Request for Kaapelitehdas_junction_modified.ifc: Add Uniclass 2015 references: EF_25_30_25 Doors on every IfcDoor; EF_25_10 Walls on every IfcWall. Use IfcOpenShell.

First a look at what the model holds.

```python
import ifcopenshell

model = ifcopenshell.open("Kaapelitehdas_junction_modified.ifc")
print(model.schema)
print("classifications:", [c.Name for c in model.by_type("IfcClassification")])
for ifc_class in ("IfcDoor", "IfcRoof", "IfcStair", "IfcWall", "IfcWindow"):
    print(ifc_class, len(model.by_type(ifc_class)))
```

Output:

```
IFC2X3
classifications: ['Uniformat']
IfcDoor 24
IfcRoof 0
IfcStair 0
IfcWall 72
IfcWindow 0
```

```python
import ifcopenshell
import ifcopenshell.api.classification

model = ifcopenshell.open("Kaapelitehdas_junction_modified.ifc")

# IFC2X3 requires Source and Edition and has no link from the project to the system.
system = model.create_entity("IfcClassification", Source="NBS", Edition="2015", Name="Uniclass 2015")

codes = {
    "IfcDoor": ("EF_25_30_25", "Doors"),
    "IfcWall": ("EF_25_10", "Walls"),
}
for ifc_class, (code, name) in codes.items():
    products = model.by_type(ifc_class)
    ifcopenshell.api.classification.add_reference(
        model, products=products, classification=system, identification=code, name=name
    )
    print(code, len(products))

model.write("Kaapelitehdas_junction_modified_v2.ifc")
```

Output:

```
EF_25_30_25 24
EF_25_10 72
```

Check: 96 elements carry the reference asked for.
